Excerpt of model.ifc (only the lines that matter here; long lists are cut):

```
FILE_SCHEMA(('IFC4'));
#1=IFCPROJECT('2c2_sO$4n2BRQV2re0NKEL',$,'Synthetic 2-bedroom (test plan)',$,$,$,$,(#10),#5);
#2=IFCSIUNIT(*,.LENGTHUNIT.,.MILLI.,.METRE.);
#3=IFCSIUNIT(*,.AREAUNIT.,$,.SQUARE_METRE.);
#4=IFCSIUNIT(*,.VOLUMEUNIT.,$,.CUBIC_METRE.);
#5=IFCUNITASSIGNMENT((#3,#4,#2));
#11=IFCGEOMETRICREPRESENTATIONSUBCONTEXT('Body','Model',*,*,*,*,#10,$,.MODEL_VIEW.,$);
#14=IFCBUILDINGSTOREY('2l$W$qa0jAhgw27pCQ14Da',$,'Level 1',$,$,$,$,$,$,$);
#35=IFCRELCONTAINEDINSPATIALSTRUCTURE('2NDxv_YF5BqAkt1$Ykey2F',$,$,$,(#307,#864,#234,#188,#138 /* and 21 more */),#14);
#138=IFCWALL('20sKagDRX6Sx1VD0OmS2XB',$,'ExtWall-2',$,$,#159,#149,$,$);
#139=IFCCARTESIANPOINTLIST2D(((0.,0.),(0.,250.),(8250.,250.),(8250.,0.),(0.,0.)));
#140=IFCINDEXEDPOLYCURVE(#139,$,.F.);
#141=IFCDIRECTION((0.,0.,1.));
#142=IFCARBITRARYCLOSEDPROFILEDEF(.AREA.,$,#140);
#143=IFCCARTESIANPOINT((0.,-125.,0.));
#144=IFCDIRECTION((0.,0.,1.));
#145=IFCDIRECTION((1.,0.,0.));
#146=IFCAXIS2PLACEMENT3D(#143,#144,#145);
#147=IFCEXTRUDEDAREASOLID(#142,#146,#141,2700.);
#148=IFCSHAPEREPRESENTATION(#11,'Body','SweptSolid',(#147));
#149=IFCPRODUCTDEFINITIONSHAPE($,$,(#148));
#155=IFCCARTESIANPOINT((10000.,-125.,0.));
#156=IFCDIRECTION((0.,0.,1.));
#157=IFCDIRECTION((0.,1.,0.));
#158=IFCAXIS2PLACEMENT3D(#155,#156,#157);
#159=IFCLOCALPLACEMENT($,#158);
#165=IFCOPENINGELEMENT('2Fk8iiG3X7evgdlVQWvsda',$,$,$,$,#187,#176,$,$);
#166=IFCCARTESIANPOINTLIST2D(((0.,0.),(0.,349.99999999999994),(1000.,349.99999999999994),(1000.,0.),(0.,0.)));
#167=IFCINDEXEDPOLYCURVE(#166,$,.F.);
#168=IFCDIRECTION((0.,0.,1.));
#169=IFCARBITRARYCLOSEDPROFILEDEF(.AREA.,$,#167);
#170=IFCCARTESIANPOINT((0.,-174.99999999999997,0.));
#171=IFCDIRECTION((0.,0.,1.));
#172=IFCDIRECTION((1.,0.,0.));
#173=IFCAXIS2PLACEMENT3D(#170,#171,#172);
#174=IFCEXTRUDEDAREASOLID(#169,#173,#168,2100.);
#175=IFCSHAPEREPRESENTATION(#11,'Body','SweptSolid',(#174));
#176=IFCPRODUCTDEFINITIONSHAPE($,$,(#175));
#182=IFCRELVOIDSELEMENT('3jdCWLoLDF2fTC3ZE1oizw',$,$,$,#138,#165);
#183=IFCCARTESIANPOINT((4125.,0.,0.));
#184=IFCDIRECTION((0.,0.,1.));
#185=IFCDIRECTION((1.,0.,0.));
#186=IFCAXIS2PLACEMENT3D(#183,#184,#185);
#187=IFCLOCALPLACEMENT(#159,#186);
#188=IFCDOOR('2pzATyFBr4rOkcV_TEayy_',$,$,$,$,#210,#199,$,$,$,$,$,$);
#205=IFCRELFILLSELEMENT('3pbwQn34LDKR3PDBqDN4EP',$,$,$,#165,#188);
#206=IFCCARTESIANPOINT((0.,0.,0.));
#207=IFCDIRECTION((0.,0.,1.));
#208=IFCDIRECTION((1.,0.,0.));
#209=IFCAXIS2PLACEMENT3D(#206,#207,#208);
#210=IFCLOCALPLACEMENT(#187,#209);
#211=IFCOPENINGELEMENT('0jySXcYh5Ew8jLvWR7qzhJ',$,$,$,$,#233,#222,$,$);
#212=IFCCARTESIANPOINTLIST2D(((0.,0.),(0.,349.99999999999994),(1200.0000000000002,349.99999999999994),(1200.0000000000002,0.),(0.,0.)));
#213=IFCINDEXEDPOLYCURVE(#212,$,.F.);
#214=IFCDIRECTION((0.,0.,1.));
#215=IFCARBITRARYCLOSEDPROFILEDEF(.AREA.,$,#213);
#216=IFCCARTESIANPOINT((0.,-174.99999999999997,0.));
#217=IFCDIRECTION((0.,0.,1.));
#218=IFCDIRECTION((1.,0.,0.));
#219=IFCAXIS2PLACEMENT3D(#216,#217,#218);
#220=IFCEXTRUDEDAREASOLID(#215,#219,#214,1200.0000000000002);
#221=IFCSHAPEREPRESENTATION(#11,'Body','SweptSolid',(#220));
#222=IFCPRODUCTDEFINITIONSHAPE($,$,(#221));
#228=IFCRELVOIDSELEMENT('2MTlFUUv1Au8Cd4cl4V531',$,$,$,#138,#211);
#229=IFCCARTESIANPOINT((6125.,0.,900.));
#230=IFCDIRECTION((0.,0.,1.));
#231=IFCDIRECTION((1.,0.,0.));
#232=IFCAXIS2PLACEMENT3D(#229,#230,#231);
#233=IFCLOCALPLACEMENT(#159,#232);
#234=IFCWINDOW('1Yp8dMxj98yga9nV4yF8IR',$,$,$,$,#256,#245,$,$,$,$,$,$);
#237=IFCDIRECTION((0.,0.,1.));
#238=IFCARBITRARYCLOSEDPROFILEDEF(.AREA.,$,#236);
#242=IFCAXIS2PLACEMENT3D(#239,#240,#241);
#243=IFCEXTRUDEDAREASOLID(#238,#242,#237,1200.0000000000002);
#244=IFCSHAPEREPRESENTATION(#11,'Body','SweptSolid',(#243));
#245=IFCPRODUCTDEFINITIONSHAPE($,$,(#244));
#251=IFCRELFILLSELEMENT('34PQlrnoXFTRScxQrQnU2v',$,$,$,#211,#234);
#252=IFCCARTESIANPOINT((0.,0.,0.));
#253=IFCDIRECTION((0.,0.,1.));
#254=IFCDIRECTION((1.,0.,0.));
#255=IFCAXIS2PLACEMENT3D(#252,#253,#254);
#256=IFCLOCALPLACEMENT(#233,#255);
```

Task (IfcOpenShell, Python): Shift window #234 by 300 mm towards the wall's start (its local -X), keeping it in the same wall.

```python
import ifcopenshell
import ifcopenshell.api.geometry
import ifcopenshell.util.placement
import ifcopenshell.util.unit

model = ifcopenshell.open("model.ifc")
unit_scale = ifcopenshell.util.unit.calculate_unit_scale(model)

window = model.by_guid("1Yp8dMxj98yga9nV4yF8IR")
opening = window.FillsVoids[0].RelatingOpeningElement
wall = opening.VoidsElements[0].RelatingBuildingElement

wall_matrix = ifcopenshell.util.placement.get_local_placement(wall.ObjectPlacement)
shift = wall_matrix[:3, 0] * -0.3 / unit_scale
before = ifcopenshell.util.placement.get_local_placement(window.ObjectPlacement)[:3, 3].copy()

# The window is placed relative to its opening, so it follows when the opening moves.
matrix = ifcopenshell.util.placement.get_local_placement(opening.ObjectPlacement)
matrix[:3, 3] += shift
ifcopenshell.api.geometry.edit_object_placement(
    model, product=opening, matrix=matrix, is_si=False, should_transform_children=True
)

after = ifcopenshell.util.placement.get_local_placement(window.ObjectPlacement)[:3, 3]
print("window moved by", (after - before).round(3) + 0.0)

model.write("model_rev.ifc")
```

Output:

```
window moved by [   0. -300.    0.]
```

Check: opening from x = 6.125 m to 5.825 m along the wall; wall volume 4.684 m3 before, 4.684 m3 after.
